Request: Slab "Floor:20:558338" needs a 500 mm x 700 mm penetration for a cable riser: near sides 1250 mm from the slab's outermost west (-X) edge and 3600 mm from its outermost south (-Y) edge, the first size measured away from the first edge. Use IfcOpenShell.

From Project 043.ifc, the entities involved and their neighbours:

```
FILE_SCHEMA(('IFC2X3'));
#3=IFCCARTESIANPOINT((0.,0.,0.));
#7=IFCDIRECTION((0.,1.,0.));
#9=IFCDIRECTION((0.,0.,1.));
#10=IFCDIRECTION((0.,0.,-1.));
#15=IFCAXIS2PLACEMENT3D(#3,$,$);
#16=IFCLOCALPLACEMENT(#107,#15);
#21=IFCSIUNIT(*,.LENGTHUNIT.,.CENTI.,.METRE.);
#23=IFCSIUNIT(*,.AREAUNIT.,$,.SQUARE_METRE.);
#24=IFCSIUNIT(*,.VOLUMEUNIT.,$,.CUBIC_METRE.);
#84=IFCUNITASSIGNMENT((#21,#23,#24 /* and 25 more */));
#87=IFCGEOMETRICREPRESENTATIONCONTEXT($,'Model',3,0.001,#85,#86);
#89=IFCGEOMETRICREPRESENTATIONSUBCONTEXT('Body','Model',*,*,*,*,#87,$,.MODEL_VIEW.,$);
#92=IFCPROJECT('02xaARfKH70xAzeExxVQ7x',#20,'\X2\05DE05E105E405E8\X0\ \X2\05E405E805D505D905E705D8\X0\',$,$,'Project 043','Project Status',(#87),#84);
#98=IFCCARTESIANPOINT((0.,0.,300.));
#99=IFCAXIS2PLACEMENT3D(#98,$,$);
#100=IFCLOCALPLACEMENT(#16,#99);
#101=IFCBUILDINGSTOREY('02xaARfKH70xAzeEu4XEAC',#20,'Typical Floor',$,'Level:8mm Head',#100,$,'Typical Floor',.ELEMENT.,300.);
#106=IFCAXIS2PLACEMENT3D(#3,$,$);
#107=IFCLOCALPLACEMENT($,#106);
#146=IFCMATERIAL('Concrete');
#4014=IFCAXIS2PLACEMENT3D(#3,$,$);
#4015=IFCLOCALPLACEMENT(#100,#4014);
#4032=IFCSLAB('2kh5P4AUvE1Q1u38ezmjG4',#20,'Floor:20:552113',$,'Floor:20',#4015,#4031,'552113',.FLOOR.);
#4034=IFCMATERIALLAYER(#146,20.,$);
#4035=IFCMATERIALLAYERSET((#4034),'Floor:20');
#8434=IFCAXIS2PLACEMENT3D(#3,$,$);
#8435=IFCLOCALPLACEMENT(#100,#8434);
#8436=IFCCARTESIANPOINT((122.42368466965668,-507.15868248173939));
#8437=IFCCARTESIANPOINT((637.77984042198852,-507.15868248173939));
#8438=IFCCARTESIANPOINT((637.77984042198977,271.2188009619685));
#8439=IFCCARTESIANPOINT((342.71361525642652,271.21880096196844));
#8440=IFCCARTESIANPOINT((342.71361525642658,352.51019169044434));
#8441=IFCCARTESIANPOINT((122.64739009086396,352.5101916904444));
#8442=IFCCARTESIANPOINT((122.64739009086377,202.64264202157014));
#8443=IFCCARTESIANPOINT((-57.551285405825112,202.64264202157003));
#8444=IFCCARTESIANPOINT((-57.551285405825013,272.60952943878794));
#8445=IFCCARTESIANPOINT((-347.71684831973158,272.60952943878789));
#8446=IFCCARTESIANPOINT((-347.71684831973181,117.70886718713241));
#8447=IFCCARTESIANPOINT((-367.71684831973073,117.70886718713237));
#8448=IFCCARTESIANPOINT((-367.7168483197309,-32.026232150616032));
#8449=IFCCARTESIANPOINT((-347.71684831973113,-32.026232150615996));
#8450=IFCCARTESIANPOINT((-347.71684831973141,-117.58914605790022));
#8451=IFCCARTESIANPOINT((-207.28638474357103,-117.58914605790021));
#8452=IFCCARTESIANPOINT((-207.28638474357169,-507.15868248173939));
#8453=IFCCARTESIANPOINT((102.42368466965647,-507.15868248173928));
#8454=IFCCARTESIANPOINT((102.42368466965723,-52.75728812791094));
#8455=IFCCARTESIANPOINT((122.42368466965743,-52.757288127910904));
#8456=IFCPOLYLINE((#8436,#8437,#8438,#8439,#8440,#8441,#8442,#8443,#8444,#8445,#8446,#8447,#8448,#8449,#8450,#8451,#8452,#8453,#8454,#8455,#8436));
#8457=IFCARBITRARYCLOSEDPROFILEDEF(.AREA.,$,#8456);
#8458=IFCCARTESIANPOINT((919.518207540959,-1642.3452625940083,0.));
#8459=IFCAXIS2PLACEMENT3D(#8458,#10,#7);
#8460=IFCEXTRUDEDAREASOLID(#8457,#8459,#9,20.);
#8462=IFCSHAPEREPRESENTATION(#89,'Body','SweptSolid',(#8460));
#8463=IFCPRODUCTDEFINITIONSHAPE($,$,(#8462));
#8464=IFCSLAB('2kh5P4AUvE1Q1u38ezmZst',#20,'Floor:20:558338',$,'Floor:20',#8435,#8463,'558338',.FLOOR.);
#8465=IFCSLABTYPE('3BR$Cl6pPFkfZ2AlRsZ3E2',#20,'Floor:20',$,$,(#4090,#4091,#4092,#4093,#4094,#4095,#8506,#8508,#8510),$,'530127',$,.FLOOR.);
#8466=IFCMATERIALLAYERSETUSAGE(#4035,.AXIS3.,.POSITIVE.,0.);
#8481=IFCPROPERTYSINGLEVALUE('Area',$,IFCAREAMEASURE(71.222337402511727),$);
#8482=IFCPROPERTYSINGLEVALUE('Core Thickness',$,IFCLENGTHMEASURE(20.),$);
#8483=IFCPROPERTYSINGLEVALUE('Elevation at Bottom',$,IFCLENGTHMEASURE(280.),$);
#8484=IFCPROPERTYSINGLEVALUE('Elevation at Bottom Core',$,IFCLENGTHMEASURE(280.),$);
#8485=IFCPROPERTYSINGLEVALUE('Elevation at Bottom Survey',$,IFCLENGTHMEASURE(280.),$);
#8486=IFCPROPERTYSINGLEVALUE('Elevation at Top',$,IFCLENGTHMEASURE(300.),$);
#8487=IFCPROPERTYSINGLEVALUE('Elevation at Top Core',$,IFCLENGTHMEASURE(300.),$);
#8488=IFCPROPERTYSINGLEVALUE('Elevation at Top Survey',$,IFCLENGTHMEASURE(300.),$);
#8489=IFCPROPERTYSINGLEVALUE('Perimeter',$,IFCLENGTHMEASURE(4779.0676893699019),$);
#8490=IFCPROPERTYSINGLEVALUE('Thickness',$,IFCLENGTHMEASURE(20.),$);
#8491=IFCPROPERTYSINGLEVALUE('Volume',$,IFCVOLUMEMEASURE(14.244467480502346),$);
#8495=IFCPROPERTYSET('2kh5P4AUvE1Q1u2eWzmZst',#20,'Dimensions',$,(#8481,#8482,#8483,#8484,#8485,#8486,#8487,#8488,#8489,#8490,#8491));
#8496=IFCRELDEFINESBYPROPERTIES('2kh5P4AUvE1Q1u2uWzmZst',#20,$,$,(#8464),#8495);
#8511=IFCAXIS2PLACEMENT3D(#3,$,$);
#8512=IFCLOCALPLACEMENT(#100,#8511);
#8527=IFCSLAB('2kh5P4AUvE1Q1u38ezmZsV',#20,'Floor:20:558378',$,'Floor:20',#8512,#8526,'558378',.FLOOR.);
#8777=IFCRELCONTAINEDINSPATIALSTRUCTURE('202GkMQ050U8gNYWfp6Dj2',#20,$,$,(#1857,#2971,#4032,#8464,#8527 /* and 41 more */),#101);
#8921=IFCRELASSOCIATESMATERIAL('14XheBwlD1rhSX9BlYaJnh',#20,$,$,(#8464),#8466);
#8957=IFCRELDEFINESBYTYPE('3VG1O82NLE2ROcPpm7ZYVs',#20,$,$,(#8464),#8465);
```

```python
import numpy as np
import ifcopenshell
import ifcopenshell.api.feature
import ifcopenshell.api.geometry
import ifcopenshell.api.pset
import ifcopenshell.api.root
import ifcopenshell.geom
import ifcopenshell.util.element
import ifcopenshell.util.placement
import ifcopenshell.util.representation
import ifcopenshell.util.shape
import ifcopenshell.util.unit

model = ifcopenshell.open("Project 043.ifc")
unit_scale = ifcopenshell.util.unit.calculate_unit_scale(model)
area_scale = ifcopenshell.util.unit.calculate_unit_scale(model, "AREAUNIT")
volume_scale = ifcopenshell.util.unit.calculate_unit_scale(model, "VOLUMEUNIT")
settings = ifcopenshell.geom.settings()


def volume(element):
    """Net volume in cubic metres, openings subtracted."""
    shape = ifcopenshell.geom.create_shape(settings, element)
    return ifcopenshell.util.shape.get_volume(shape.geometry)


slab = model.by_id(8464)
before = volume(slab)

# Extent in the slab's own axes, in metres. The edges named are its -X and -Y sides.
slab_shape = ifcopenshell.geom.create_shape(settings, slab)
vertices = ifcopenshell.util.shape.get_vertices(slab_shape.geometry)
x_min, y_min, bottom = vertices.min(axis=0)
top = vertices[:, 2].max()

opening = ifcopenshell.api.root.create_entity(model, ifc_class="IfcOpeningElement", name="Cable riser opening")
context = ifcopenshell.util.representation.get_context(model, "Model", "Body", "MODEL_VIEW")
width, depth = 0.5, 0.7
outline = [(0.0, 0.0), (width, 0.0), (width, depth), (0.0, depth), (0.0, 0.0)]
# Overshoot both faces by 50 mm so the cut is clean.
shape = ifcopenshell.api.geometry.add_slab_representation(
    model, context=context, depth=top - bottom + 0.1, polyline=outline
)
ifcopenshell.api.geometry.assign_representation(model, product=opening, representation=shape)

matrix = ifcopenshell.util.placement.get_local_placement(slab.ObjectPlacement)
matrix[:, 3] = matrix @ np.append(np.array([x_min + 1.25, y_min + 3.6, bottom - 0.05]) / unit_scale, 1.0)
ifcopenshell.api.geometry.edit_object_placement(model, product=opening, matrix=matrix, is_si=False)
ifcopenshell.api.feature.add_feature(model, feature=opening, element=slab)

after = volume(slab)

# Update the slab's stored quantities.
pset = model.by_id(ifcopenshell.util.element.get_pset(slab, "Dimensions", should_inherit=False)["id"])
ifcopenshell.api.pset.edit_pset(model, pset=pset, properties={
    "Area": model.create_entity("IfcAreaMeasure", after / (top - bottom) / area_scale),
    "Volume": model.create_entity("IfcVolumeMeasure", after / volume_scale),
})

print(f"slab volume {before:.3f} -> {after:.3f} m3")

model.write("Project 043_edited.ifc")
```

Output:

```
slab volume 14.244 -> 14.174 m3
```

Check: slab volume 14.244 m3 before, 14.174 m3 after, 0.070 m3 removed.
